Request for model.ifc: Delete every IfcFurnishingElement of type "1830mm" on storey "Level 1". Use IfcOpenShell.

First a look at what the model holds.

```python
import ifcopenshell
import ifcopenshell.util.element

model = ifcopenshell.open("model.ifc")
print(model.schema)
storey = next(s for s in model.by_type("IfcBuildingStorey") if s.Name == "Level 1")
furniture = [e for e in ifcopenshell.util.element.get_decomposition(storey) if e.is_a("IfcFurnishingElement")]
seen = {}
for e in furniture:
    element_type = ifcopenshell.util.element.get_type(e)
    name = element_type.Name if element_type not in (None, e) else None
    seen[name] = seen.get(name, 0) + 1
for name, count in sorted(seen.items(), key=str):
    print(count, "x", name)
```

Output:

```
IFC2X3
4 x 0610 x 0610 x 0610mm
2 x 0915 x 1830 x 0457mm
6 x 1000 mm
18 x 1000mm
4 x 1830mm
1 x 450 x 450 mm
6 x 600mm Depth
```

```python
import ifcopenshell
import ifcopenshell.api.root
import ifcopenshell.util.element

model = ifcopenshell.open("model.ifc")

storey = next(s for s in model.by_type("IfcBuildingStorey") if s.Name == "Level 1")
furniture = [e for e in ifcopenshell.util.element.get_decomposition(storey) if e.is_a("IfcFurnishingElement")]
targets = [e for e in furniture if (t := ifcopenshell.util.element.get_type(e)) not in (None, e) and t.Name == "1830mm"]

for e in targets:
    ifcopenshell.api.root.remove_product(model, product=e)
print(len(targets), "removed")

model.write("model_v2.ifc")
```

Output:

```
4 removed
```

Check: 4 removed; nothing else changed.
